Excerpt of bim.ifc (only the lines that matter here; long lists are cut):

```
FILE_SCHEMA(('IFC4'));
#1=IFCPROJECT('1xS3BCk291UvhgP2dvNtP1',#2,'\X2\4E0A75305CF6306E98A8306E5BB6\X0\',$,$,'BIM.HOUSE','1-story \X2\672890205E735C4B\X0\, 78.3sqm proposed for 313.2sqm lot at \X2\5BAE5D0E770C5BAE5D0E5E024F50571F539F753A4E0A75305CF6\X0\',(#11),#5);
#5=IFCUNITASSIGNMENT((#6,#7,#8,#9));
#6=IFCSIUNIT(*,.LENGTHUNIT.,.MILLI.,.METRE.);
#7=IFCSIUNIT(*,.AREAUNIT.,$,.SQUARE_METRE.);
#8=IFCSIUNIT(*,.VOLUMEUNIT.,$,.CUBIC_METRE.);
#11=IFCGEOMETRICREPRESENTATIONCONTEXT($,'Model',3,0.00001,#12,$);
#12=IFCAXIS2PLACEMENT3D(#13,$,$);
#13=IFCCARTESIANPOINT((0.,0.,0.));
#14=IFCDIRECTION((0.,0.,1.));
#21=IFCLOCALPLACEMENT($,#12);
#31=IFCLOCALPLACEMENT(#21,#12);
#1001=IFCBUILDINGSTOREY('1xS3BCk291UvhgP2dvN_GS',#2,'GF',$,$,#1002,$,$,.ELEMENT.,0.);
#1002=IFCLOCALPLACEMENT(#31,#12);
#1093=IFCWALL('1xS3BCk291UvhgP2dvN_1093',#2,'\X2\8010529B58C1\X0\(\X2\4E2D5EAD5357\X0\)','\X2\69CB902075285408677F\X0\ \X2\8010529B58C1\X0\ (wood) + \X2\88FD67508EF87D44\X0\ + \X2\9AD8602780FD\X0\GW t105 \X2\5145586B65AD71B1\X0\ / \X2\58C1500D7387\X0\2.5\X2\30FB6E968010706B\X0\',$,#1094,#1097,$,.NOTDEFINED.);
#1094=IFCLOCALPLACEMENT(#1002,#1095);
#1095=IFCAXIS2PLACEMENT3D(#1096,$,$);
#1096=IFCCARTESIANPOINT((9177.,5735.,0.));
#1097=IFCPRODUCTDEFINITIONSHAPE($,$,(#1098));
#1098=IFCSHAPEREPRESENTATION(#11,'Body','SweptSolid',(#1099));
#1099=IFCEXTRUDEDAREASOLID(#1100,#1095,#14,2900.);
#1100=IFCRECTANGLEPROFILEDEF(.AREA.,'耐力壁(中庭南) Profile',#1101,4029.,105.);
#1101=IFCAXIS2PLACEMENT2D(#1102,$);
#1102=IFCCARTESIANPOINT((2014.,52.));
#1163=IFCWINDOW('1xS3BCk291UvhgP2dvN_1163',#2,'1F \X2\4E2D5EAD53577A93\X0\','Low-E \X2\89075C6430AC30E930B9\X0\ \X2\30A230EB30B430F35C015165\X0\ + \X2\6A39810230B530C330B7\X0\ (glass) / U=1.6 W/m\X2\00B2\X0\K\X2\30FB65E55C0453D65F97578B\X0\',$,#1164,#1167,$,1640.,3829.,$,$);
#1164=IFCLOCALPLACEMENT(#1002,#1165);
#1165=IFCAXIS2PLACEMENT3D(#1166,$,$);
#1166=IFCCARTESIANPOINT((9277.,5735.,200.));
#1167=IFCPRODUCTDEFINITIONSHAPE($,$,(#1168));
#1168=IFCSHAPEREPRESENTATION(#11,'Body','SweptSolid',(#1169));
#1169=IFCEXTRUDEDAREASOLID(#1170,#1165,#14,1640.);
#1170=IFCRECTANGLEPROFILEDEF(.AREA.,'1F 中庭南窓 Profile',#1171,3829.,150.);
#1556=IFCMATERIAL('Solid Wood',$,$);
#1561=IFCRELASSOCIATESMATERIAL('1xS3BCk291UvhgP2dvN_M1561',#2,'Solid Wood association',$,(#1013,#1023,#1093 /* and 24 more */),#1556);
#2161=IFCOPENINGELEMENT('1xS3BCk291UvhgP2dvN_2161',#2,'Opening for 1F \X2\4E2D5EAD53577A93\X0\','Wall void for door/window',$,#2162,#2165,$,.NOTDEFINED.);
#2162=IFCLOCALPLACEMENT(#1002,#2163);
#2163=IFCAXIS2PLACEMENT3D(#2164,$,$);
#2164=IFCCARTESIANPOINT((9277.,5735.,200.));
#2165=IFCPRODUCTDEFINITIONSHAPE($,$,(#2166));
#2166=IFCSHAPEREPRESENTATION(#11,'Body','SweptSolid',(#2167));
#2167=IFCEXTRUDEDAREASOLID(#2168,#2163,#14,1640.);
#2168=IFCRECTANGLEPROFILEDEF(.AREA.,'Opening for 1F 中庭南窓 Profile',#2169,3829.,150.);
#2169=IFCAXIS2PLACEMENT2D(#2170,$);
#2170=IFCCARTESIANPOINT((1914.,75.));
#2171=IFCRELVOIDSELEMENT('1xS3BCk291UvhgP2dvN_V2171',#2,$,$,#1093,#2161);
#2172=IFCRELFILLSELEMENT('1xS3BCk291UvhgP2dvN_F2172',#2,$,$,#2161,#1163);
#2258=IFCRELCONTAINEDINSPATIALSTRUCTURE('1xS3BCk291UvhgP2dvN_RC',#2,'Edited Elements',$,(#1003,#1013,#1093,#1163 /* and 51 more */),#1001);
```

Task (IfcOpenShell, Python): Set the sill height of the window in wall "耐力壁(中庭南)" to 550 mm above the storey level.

```python
import numpy as np
import ifcopenshell
import ifcopenshell.api.geometry
import ifcopenshell.geom
import ifcopenshell.util.element
import ifcopenshell.util.placement
import ifcopenshell.util.shape
import ifcopenshell.util.unit

model = ifcopenshell.open("bim.ifc")
unit_scale = ifcopenshell.util.unit.calculate_unit_scale(model)

window = model.by_guid("1xS3BCk291UvhgP2dvN_1163")
opening = window.FillsVoids[0].RelatingOpeningElement
storey = ifcopenshell.util.element.get_container(window, ifc_class="IfcBuildingStorey")
level = ifcopenshell.util.placement.get_local_placement(storey.ObjectPlacement)[2, 3]

# The opening's origin need not be at the sill, so measure its lowest point.
shape = ifcopenshell.geom.create_shape(ifcopenshell.geom.settings(), opening)
bottom = ifcopenshell.util.shape.get_shape_bottom_elevation(shape, shape.geometry) / unit_scale
dz = level + 0.55 / unit_scale - bottom

shift = np.array([0.0, 0.0, dz])
# The window is not placed relative to its opening, so move both.
for product in (opening, window):
    matrix = ifcopenshell.util.placement.get_local_placement(product.ObjectPlacement)
    matrix[:3, 3] += shift
    ifcopenshell.api.geometry.edit_object_placement(model, product=product, matrix=matrix, is_si=False)

print(f"moved by {dz * unit_scale:+.3f} m")

model.write("bim_rev.ifc")
```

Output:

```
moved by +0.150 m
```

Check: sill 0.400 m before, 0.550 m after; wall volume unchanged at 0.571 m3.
